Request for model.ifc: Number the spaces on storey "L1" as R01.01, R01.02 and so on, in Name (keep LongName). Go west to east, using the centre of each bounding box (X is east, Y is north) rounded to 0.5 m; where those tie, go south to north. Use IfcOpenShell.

First a look at what the model holds.

```python
import ifcopenshell
import ifcopenshell.util.element
import ifcopenshell.util.placement

model = ifcopenshell.open("model.ifc")
print(model.schema)
storey = next(s for s in model.by_type("IfcBuildingStorey") if s.Name == "L1")
spaces = [e for e in ifcopenshell.util.element.get_decomposition(storey) if e.is_a("IfcSpace")]
for e in sorted(spaces, key=lambda e: e.id()):
    origin = ifcopenshell.util.placement.get_local_placement(e.ObjectPlacement)[:3, 3]
    print(e.id(), e.Name, e.LongName, origin.round(2) + 0.0, sep=" | ")
```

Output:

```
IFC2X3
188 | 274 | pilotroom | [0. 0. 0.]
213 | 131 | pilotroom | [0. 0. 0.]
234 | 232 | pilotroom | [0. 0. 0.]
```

```python
import ifcopenshell
import ifcopenshell.geom
import ifcopenshell.util.element
import ifcopenshell.util.shape

model = ifcopenshell.open("model.ifc")
settings = ifcopenshell.geom.settings()
settings.set("use-world-coords", True)


def centre(element):
    shape = ifcopenshell.geom.create_shape(settings, element)
    return ifcopenshell.util.shape.get_bbox_centroid(shape.geometry)


storey = next(s for s in model.by_type("IfcBuildingStorey") if s.Name == "L1")
spaces = [e for e in ifcopenshell.util.element.get_decomposition(storey) if e.is_a("IfcSpace")]

# Insertion points can sit at a corner or the storey origin, so sort by the geometry (in metres).
centres = {e: centre(e) for e in spaces}
spaces.sort(key=lambda e: (round(centres[e][0] / 0.5), centres[e][1]))

for i, e in enumerate(spaces, start=1):
    number = f"R01.{i:02d}"
    e.Name = number
    print(e.id(), number)

model.write("model_updated.ifc")
```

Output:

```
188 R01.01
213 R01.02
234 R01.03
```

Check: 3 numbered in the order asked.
